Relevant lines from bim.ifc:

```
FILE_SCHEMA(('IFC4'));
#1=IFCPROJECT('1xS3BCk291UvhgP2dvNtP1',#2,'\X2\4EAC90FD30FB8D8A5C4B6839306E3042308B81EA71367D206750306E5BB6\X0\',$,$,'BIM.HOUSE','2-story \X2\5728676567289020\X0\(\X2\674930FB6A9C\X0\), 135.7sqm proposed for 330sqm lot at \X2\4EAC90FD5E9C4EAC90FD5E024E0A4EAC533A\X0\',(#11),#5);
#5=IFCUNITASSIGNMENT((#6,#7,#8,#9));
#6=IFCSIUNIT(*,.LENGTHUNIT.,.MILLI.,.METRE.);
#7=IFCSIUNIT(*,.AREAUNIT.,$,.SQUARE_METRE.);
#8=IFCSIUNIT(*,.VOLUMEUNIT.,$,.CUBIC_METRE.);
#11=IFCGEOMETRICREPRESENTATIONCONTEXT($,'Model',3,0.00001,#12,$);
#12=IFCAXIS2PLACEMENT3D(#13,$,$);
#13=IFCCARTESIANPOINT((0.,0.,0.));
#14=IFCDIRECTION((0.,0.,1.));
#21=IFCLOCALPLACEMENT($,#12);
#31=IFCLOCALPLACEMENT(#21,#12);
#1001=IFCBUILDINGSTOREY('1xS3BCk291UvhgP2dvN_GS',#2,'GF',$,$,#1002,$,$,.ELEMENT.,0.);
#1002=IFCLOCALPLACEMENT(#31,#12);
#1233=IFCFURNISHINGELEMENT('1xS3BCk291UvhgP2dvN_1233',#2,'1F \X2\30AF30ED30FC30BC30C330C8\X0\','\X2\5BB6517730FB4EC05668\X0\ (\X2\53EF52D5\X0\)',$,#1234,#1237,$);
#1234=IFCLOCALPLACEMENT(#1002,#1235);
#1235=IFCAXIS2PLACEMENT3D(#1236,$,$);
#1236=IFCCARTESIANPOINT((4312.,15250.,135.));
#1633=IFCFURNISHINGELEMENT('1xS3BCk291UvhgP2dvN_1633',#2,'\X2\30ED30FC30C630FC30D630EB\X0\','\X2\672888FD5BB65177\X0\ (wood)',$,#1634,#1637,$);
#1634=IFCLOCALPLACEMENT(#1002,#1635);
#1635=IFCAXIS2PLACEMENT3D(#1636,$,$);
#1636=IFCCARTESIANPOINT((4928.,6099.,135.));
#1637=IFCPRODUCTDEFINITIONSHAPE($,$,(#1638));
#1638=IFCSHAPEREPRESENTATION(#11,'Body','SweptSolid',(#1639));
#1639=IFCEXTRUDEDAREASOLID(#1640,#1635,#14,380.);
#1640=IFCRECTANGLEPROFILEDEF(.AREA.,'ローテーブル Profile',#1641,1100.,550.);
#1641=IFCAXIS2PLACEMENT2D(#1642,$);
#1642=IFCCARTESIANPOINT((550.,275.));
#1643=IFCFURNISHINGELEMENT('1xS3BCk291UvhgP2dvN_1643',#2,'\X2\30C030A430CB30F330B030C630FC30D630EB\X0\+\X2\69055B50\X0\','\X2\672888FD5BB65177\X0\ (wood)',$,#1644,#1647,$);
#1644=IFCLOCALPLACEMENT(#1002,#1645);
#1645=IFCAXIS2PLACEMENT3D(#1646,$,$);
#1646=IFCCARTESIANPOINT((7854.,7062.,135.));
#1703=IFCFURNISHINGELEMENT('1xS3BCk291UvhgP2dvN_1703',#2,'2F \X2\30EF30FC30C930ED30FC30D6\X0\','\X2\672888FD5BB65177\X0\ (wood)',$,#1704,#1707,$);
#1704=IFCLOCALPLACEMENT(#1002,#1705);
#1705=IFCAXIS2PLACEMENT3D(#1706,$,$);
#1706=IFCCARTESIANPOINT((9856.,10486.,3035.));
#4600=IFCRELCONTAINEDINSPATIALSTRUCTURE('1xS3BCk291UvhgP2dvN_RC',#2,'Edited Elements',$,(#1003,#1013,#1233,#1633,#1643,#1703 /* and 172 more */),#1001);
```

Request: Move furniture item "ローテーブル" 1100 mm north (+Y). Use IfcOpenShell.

```python
import ifcopenshell
import ifcopenshell.api.geometry
import ifcopenshell.util.placement

model = ifcopenshell.open("bim.ifc")

item = model.by_id(1633)
matrix = ifcopenshell.util.placement.get_local_placement(item.ObjectPlacement)
matrix[1, 3] += 1100.0
ifcopenshell.api.geometry.edit_object_placement(model, product=item, matrix=matrix, is_si=False)

print(ifcopenshell.util.placement.get_local_placement(item.ObjectPlacement).round(3) + 0.0)

model.write("bim_rev.ifc")
```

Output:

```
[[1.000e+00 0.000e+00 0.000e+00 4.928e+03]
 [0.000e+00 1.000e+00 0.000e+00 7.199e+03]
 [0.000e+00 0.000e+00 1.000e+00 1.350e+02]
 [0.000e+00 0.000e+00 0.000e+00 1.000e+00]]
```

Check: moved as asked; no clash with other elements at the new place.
